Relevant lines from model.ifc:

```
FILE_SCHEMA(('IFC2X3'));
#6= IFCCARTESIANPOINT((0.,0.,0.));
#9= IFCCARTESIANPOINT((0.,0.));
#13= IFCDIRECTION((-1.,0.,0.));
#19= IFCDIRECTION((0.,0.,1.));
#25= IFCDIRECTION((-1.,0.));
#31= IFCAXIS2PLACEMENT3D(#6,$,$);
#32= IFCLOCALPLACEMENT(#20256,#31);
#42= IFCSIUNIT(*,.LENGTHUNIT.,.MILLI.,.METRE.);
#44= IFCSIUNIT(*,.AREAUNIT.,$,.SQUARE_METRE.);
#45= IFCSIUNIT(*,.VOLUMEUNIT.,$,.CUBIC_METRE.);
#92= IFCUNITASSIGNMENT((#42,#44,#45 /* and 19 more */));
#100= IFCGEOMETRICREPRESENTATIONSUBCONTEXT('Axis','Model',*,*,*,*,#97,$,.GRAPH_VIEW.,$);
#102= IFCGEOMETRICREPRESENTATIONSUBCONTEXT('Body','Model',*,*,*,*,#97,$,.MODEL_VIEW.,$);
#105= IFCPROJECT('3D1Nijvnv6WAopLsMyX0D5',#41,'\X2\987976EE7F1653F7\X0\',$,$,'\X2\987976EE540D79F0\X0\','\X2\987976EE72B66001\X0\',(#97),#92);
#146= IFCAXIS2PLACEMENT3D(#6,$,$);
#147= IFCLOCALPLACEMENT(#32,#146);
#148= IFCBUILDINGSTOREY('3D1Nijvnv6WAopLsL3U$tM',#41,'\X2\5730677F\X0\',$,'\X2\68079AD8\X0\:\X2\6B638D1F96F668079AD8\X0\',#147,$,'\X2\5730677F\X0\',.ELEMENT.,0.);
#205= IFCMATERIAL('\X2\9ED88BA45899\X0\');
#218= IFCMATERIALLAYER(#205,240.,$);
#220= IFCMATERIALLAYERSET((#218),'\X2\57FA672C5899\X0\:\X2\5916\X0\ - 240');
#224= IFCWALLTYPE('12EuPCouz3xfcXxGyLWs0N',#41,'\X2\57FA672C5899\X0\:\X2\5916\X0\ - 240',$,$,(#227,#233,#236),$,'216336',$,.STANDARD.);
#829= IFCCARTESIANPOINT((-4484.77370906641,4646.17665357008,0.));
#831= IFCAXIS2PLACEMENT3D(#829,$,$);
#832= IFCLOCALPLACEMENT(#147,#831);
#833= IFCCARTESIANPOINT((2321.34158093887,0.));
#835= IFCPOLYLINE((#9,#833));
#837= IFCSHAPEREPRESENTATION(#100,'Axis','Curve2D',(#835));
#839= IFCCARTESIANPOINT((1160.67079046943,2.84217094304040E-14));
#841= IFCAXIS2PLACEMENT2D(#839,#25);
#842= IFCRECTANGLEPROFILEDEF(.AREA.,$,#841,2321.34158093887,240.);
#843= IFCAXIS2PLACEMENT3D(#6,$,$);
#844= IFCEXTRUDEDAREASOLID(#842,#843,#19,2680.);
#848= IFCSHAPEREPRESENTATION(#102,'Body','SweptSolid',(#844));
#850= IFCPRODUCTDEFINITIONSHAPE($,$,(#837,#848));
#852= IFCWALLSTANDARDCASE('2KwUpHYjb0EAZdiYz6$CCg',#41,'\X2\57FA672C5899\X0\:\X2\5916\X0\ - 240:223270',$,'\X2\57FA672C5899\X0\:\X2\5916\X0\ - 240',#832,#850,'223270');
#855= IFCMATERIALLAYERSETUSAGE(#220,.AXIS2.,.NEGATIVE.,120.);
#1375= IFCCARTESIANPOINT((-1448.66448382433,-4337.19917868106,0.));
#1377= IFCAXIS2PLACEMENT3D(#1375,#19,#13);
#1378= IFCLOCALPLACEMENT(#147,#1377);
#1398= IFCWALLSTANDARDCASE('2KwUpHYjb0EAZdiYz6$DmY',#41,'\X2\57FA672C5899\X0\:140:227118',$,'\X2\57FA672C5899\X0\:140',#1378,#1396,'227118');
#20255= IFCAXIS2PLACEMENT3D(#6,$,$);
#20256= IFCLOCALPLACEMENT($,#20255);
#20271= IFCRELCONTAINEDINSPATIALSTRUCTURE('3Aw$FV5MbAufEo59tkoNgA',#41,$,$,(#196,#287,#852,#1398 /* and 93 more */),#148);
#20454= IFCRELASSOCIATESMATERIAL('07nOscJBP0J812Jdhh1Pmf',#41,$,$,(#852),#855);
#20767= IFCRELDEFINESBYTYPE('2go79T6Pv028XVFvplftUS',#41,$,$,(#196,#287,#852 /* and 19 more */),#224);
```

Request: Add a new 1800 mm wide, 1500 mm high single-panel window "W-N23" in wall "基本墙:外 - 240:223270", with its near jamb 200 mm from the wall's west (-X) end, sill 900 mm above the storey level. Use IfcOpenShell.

```python
import numpy as np
import ifcopenshell
import ifcopenshell.api.feature
import ifcopenshell.api.geometry
import ifcopenshell.api.root
import ifcopenshell.api.spatial
import ifcopenshell.api.type
import ifcopenshell.geom
import ifcopenshell.util.element
import ifcopenshell.util.placement
import ifcopenshell.util.representation
import ifcopenshell.util.shape
import ifcopenshell.util.unit

model = ifcopenshell.open("model.ifc")
unit_scale = ifcopenshell.util.unit.calculate_unit_scale(model)
settings = ifcopenshell.geom.settings()


def volume(element):
    """Net volume in cubic metres, openings subtracted."""
    shape = ifcopenshell.geom.create_shape(settings, element)
    return ifcopenshell.util.shape.get_volume(shape.geometry)


wall = model.by_guid("2KwUpHYjb0EAZdiYz6$CCg")
storey = ifcopenshell.util.element.get_container(wall, ifc_class="IfcBuildingStorey")
context = ifcopenshell.util.representation.get_context(model, "Model", "Body", "MODEL_VIEW")
before = volume(wall)

width, height, from_end, sill = 1.8, 1.5, 0.2, 0.9  # metres

# The wall runs along its own X axis, and the end named is its -X end.
wall_shape = ifcopenshell.geom.create_shape(settings, wall)
x, y, z = ifcopenshell.util.shape.get_vertices(wall_shape.geometry).T
start = x.min() + from_end
face, thickness = float(y.min()), float(y.max() - y.min())
wall_matrix = ifcopenshell.util.placement.get_local_placement(wall.ObjectPlacement)
level = ifcopenshell.util.placement.get_local_placement(storey.ObjectPlacement)[2, 3]


def in_wall(x, y):
    """Placement at x, y metres in the wall's axes, at sill height."""
    matrix = wall_matrix.copy()
    matrix[:, 3] = wall_matrix @ np.array([x / unit_scale, y / unit_scale, 0.0, 1.0])
    matrix[2, 3] = level + sill / unit_scale
    return matrix


# Opening: a box that overshoots both wall faces by 50 mm.
opening = ifcopenshell.api.root.create_entity(model, ifc_class="IfcOpeningElement")
box = ifcopenshell.api.geometry.add_wall_representation(
    model, context=context, length=width, height=height, thickness=thickness + 0.1
)
ifcopenshell.api.geometry.assign_representation(model, product=opening, representation=box)
ifcopenshell.api.geometry.edit_object_placement(model, product=opening, matrix=in_wall(start, face - 0.05), is_si=False)
ifcopenshell.api.feature.add_feature(model, feature=opening, element=wall)

window = ifcopenshell.api.root.create_entity(model, ifc_class="IfcWindow", name="W-N23")
window.OverallWidth, window.OverallHeight = width / unit_scale, height / unit_scale
body = ifcopenshell.api.geometry.add_window_representation(
    model,
    context=context,
    overall_width=window.OverallWidth,
    overall_height=window.OverallHeight,
    partition_type="SINGLE_PANEL",
)
ifcopenshell.api.geometry.assign_representation(model, product=window, representation=body)
ifcopenshell.api.spatial.assign_container(model, products=[window], relating_structure=storey)
fills = ifcopenshell.api.feature.add_filling(model, opening=opening, element=window)
fills.OwnerHistory = window.OwnerHistory  # required in IFC2X3

# IFC2X3 keeps the operation on the window style.
style = ifcopenshell.api.root.create_entity(model, ifc_class="IfcWindowStyle", name="W-N23")
style.OperationType, style.ConstructionType = "SINGLE_PANEL", "NOTDEFINED"
style.ParameterTakesPrecedence = style.Sizeable = False
ifcopenshell.api.type.assign_type(model, related_objects=[window], relating_type=style)

# Centre the window in the wall's thickness.
ifcopenshell.api.geometry.edit_object_placement(model, product=window, matrix=in_wall(start, face), is_si=False)
window_shape = ifcopenshell.geom.create_shape(settings, window)
depth = ifcopenshell.util.shape.get_vertices(window_shape.geometry)[:, 1]
offset = face + thickness / 2 - (depth.min() + depth.max()) / 2
ifcopenshell.api.geometry.edit_object_placement(model, product=window, matrix=in_wall(start, offset), is_si=False)

after = volume(wall)

print(f"wall volume {before:.3f} -> {after:.3f} m3")

model.write("model-out.ifc")
```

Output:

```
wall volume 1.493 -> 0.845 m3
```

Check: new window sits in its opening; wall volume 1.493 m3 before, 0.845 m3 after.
